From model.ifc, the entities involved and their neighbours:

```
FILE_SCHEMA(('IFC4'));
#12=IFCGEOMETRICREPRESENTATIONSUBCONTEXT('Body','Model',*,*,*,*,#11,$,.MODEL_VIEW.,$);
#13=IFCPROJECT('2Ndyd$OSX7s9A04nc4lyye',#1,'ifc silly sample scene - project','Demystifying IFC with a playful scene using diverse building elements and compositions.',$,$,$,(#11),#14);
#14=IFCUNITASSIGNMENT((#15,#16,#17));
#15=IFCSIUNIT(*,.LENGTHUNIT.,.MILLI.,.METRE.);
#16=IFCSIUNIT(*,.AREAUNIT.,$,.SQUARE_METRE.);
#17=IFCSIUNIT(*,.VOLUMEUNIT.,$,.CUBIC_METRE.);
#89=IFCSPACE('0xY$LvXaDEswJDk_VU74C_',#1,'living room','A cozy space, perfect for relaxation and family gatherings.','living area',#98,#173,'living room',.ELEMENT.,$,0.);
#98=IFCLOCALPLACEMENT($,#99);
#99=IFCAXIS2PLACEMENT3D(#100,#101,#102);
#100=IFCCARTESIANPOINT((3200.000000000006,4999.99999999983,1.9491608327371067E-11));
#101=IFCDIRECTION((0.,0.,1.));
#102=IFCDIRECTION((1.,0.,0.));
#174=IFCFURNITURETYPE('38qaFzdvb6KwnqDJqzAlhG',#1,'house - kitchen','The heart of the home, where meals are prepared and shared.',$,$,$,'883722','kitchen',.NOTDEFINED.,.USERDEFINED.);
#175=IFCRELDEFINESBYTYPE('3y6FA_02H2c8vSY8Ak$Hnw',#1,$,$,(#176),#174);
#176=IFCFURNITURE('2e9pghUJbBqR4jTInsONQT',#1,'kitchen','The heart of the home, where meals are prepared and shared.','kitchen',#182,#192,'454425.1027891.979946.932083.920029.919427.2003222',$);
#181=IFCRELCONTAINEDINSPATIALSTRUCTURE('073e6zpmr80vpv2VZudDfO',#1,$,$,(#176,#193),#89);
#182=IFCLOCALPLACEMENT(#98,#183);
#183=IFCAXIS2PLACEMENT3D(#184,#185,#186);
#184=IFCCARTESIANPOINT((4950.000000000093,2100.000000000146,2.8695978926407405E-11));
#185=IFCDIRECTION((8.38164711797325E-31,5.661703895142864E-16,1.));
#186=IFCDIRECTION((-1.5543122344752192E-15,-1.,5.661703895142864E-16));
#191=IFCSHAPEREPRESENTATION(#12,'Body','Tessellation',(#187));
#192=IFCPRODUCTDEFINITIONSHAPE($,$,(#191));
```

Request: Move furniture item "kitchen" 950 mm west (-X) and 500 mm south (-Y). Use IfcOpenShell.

```python
import ifcopenshell
import ifcopenshell.api.geometry
import ifcopenshell.util.placement
import ifcopenshell.util.unit

model = ifcopenshell.open("model.ifc")
unit_scale = ifcopenshell.util.unit.calculate_unit_scale(model)

item = model.by_guid("2e9pghUJbBqR4jTInsONQT")
matrix = ifcopenshell.util.placement.get_local_placement(item.ObjectPlacement)
matrix[0, 3] -= 0.95 / unit_scale
matrix[1, 3] -= 0.5 / unit_scale
ifcopenshell.api.geometry.edit_object_placement(model, product=item, matrix=matrix, is_si=False)

print(ifcopenshell.util.placement.get_local_placement(item.ObjectPlacement).round(3) + 0.0)

model.write("model_rev.ifc")
```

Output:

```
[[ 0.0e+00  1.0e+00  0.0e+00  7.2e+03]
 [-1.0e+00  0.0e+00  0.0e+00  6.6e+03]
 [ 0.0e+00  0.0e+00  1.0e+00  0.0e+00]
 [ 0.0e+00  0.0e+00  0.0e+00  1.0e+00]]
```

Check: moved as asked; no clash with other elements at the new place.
